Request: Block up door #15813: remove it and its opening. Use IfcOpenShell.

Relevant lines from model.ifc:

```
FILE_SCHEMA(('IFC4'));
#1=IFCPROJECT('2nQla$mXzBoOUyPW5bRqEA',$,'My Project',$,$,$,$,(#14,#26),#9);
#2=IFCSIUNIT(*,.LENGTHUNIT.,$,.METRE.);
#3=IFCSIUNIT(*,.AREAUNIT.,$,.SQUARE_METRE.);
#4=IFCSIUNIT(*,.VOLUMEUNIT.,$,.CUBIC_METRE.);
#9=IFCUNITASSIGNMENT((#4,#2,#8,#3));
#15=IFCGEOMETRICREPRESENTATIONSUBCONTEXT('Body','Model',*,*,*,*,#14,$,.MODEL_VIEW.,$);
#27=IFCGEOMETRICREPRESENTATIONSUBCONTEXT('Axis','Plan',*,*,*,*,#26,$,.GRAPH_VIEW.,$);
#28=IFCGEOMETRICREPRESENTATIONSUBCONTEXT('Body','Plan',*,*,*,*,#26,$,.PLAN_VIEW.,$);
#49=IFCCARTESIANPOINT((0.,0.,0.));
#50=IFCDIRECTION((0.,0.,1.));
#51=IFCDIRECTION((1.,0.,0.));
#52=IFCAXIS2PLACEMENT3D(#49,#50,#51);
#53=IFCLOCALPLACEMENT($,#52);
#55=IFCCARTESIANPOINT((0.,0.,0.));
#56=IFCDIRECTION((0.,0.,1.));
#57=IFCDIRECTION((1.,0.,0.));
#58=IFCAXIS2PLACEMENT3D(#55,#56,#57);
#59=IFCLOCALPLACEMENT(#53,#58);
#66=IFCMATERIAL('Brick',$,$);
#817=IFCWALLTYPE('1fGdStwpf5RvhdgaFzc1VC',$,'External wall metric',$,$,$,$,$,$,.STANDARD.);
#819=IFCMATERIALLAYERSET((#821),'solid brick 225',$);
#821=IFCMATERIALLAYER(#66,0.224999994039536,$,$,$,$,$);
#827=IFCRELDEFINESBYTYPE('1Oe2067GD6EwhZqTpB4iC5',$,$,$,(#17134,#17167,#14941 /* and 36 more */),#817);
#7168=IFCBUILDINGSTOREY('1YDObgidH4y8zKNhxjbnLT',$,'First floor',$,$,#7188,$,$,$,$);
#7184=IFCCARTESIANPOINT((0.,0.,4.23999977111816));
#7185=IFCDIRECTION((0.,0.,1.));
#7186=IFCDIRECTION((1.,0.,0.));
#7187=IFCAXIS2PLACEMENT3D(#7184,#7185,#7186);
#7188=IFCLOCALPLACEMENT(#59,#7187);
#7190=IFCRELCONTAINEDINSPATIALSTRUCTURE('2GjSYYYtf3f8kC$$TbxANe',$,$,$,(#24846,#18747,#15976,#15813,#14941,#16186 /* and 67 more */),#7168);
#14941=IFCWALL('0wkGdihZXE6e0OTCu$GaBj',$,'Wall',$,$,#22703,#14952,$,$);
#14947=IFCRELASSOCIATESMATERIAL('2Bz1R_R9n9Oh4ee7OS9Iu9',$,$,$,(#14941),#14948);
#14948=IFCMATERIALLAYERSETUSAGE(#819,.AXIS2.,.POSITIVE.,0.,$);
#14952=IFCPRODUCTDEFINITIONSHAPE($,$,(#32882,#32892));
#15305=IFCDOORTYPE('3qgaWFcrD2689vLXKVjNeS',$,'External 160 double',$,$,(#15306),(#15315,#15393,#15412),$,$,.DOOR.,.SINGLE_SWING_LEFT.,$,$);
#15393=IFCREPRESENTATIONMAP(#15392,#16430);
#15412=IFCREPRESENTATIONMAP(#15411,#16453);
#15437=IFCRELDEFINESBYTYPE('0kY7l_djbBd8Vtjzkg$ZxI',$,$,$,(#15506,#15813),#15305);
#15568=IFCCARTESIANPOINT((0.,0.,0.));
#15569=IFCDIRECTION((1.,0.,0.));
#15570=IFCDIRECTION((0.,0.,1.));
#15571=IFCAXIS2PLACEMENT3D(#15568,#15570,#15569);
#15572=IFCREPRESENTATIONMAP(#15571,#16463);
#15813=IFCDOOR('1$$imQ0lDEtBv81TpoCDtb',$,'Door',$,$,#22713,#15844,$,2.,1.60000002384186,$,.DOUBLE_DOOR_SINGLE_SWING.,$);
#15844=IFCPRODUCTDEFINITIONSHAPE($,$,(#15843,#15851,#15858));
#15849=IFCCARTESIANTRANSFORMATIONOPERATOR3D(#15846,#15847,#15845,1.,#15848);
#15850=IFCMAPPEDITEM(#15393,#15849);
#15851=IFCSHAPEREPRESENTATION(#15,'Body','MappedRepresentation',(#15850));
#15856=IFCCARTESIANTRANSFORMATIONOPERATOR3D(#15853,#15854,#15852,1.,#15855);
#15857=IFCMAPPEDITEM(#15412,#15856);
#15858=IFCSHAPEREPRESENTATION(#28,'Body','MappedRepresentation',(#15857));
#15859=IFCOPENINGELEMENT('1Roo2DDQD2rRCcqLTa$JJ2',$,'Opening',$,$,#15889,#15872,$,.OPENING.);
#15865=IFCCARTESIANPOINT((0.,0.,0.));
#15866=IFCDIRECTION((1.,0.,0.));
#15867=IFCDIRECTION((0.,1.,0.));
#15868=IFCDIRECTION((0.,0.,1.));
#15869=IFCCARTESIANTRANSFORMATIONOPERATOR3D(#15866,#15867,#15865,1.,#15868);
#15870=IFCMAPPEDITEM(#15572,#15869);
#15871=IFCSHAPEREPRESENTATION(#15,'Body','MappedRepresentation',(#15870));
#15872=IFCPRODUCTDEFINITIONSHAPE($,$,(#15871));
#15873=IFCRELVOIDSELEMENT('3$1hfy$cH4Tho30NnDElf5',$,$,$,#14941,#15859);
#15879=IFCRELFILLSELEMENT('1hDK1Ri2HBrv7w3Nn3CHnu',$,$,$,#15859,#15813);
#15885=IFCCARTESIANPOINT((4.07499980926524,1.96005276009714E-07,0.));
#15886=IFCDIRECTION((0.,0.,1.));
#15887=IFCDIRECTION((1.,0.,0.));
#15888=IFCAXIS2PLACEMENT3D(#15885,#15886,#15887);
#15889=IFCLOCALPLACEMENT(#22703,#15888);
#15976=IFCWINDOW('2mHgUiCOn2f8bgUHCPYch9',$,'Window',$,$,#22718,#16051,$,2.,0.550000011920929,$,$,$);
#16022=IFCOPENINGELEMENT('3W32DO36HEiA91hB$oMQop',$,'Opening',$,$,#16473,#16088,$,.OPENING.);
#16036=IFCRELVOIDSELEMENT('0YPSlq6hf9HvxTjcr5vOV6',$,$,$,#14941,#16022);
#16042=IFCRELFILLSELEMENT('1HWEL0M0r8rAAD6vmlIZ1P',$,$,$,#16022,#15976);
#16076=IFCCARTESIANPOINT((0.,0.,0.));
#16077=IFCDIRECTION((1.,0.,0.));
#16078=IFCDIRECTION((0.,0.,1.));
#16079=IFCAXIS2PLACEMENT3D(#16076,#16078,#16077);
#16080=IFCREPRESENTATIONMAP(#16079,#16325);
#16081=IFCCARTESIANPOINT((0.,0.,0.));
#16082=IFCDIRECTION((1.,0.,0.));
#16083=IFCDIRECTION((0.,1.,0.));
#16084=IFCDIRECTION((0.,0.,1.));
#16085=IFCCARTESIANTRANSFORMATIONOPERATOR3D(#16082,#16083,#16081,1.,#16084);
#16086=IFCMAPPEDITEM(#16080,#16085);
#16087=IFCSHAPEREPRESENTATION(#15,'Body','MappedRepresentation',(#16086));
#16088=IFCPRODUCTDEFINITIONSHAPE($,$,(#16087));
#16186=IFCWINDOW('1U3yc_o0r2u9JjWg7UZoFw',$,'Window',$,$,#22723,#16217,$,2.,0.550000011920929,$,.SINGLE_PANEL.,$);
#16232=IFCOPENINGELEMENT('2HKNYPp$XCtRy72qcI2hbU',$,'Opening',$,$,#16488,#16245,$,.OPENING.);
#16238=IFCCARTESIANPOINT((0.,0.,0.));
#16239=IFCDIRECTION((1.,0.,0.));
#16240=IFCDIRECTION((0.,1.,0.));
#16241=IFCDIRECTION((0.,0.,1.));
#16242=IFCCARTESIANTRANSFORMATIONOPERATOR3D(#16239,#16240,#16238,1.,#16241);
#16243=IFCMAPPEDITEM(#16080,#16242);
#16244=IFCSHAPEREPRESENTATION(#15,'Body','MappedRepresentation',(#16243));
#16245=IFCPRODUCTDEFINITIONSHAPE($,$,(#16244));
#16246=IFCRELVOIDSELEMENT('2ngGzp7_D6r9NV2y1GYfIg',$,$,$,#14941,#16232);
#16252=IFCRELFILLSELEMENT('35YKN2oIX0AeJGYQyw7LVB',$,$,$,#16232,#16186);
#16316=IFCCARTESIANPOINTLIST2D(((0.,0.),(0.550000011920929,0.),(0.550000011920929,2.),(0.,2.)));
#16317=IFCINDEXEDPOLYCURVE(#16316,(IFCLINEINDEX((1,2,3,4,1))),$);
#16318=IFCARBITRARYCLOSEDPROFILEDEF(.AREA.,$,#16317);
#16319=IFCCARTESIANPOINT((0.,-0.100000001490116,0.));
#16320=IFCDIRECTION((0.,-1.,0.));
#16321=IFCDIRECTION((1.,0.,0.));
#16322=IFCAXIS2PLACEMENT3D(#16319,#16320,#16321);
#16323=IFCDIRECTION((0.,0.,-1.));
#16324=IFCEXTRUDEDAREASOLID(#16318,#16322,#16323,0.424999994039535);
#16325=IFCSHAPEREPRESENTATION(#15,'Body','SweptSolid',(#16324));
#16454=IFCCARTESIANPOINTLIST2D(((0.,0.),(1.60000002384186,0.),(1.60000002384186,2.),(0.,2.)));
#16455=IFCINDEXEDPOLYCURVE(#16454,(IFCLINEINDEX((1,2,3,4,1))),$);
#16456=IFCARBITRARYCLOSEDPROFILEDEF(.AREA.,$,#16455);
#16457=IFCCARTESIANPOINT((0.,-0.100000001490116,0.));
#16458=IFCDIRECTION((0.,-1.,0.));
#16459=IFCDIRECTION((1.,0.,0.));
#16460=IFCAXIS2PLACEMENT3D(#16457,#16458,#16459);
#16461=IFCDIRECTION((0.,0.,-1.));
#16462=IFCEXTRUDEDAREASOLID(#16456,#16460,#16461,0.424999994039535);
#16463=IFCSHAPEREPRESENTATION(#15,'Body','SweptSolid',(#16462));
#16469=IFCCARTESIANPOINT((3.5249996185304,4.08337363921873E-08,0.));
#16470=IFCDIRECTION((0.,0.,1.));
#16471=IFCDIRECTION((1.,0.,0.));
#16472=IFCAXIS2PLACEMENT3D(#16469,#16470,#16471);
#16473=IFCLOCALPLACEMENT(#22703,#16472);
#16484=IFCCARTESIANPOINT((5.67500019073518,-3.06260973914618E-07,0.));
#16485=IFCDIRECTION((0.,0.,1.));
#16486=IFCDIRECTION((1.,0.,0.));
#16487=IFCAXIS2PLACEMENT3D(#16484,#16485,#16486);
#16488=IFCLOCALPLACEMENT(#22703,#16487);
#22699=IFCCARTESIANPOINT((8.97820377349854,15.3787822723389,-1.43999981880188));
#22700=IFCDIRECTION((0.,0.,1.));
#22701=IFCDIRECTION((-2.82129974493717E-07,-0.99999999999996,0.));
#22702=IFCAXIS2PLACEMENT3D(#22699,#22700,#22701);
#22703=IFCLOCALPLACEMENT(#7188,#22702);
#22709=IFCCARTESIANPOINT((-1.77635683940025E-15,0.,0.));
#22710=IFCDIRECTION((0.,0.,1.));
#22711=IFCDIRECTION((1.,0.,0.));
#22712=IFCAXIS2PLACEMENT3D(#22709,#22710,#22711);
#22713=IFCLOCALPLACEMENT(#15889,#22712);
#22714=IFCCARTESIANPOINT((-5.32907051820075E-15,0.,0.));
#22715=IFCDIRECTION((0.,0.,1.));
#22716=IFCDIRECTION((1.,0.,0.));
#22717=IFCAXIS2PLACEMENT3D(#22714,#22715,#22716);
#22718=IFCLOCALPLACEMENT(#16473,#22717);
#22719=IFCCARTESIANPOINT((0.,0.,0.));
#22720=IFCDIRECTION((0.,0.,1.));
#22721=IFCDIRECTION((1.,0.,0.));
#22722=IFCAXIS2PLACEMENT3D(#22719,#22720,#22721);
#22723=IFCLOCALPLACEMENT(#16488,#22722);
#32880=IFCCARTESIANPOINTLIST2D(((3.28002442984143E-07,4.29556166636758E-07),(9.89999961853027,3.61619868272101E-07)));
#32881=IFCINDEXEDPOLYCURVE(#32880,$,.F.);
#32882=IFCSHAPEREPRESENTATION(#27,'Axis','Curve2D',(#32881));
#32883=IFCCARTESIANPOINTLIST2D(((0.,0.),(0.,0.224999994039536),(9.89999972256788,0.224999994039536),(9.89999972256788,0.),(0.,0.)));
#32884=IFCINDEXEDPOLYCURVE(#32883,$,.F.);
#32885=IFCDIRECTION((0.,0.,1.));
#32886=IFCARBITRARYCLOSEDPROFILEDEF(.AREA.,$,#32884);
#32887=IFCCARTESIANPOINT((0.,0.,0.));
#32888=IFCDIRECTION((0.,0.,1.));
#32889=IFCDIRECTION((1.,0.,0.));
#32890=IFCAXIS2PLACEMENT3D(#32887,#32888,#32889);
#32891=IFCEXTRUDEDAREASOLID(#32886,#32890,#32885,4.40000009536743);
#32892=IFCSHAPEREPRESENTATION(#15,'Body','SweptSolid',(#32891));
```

```python
import ifcopenshell
import ifcopenshell.api.feature
import ifcopenshell.api.root
import ifcopenshell.geom
import ifcopenshell.util.shape

model = ifcopenshell.open("model.ifc")
settings = ifcopenshell.geom.settings()


def volume(element):
    """Net volume in cubic metres, openings subtracted."""
    shape = ifcopenshell.geom.create_shape(settings, element)
    return ifcopenshell.util.shape.get_volume(shape.geometry)


door = model.by_id(15813)
opening = door.FillsVoids[0].RelatingOpeningElement
wall = opening.VoidsElements[0].RelatingBuildingElement
before = volume(wall)

ifcopenshell.api.root.remove_product(model, product=door)
ifcopenshell.api.feature.remove_feature(model, feature=opening)

after = volume(wall)

print(f"wall volume {before:.3f} -> {after:.3f} m3")

model.write("model_edited.ifc")
```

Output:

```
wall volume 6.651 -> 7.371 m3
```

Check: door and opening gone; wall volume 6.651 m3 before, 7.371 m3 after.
